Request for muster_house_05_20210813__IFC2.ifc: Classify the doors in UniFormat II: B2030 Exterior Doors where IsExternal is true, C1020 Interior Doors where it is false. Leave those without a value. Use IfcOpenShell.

First a look at what the model holds.

```python
import ifcopenshell
import ifcopenshell.util.element

model = ifcopenshell.open("muster_house_05_20210813__IFC2.ifc")
print(model.schema)
print("classifications:", [c.Name for c in model.by_type("IfcClassification")])
values = [ifcopenshell.util.element.get_pset(e, "Pset_DoorCommon", "IsExternal") for e in model.by_type("IfcDoor")]
for value in (True, False, None):
    print("IsExternal", value, values.count(value))
```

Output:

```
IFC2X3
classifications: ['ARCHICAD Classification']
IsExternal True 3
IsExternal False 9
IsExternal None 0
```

```python
import ifcopenshell
import ifcopenshell.api.classification
import ifcopenshell.util.element

model = ifcopenshell.open("muster_house_05_20210813__IFC2.ifc")

# IFC2X3 requires Source and Edition and has no link from the project to the system.
system = model.create_entity("IfcClassification", Source="ASTM", Edition="E1557", Name="UniFormat II")

doors = model.by_type("IfcDoor")
external = {e: ifcopenshell.util.element.get_pset(e, "Pset_DoorCommon", "IsExternal") for e in doors}
for flag, code, name in ((True, "B2030", "Exterior Doors"), (False, "C1020", "Interior Doors")):
    products = [e for e in doors if external[e] is flag]
    ifcopenshell.api.classification.add_reference(
        model, products=products, classification=system, identification=code, name=name
    )
    print(code, len(products))

model.write("muster_house_05_20210813__IFC2-out.ifc")
```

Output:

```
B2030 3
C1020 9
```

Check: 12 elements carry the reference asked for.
